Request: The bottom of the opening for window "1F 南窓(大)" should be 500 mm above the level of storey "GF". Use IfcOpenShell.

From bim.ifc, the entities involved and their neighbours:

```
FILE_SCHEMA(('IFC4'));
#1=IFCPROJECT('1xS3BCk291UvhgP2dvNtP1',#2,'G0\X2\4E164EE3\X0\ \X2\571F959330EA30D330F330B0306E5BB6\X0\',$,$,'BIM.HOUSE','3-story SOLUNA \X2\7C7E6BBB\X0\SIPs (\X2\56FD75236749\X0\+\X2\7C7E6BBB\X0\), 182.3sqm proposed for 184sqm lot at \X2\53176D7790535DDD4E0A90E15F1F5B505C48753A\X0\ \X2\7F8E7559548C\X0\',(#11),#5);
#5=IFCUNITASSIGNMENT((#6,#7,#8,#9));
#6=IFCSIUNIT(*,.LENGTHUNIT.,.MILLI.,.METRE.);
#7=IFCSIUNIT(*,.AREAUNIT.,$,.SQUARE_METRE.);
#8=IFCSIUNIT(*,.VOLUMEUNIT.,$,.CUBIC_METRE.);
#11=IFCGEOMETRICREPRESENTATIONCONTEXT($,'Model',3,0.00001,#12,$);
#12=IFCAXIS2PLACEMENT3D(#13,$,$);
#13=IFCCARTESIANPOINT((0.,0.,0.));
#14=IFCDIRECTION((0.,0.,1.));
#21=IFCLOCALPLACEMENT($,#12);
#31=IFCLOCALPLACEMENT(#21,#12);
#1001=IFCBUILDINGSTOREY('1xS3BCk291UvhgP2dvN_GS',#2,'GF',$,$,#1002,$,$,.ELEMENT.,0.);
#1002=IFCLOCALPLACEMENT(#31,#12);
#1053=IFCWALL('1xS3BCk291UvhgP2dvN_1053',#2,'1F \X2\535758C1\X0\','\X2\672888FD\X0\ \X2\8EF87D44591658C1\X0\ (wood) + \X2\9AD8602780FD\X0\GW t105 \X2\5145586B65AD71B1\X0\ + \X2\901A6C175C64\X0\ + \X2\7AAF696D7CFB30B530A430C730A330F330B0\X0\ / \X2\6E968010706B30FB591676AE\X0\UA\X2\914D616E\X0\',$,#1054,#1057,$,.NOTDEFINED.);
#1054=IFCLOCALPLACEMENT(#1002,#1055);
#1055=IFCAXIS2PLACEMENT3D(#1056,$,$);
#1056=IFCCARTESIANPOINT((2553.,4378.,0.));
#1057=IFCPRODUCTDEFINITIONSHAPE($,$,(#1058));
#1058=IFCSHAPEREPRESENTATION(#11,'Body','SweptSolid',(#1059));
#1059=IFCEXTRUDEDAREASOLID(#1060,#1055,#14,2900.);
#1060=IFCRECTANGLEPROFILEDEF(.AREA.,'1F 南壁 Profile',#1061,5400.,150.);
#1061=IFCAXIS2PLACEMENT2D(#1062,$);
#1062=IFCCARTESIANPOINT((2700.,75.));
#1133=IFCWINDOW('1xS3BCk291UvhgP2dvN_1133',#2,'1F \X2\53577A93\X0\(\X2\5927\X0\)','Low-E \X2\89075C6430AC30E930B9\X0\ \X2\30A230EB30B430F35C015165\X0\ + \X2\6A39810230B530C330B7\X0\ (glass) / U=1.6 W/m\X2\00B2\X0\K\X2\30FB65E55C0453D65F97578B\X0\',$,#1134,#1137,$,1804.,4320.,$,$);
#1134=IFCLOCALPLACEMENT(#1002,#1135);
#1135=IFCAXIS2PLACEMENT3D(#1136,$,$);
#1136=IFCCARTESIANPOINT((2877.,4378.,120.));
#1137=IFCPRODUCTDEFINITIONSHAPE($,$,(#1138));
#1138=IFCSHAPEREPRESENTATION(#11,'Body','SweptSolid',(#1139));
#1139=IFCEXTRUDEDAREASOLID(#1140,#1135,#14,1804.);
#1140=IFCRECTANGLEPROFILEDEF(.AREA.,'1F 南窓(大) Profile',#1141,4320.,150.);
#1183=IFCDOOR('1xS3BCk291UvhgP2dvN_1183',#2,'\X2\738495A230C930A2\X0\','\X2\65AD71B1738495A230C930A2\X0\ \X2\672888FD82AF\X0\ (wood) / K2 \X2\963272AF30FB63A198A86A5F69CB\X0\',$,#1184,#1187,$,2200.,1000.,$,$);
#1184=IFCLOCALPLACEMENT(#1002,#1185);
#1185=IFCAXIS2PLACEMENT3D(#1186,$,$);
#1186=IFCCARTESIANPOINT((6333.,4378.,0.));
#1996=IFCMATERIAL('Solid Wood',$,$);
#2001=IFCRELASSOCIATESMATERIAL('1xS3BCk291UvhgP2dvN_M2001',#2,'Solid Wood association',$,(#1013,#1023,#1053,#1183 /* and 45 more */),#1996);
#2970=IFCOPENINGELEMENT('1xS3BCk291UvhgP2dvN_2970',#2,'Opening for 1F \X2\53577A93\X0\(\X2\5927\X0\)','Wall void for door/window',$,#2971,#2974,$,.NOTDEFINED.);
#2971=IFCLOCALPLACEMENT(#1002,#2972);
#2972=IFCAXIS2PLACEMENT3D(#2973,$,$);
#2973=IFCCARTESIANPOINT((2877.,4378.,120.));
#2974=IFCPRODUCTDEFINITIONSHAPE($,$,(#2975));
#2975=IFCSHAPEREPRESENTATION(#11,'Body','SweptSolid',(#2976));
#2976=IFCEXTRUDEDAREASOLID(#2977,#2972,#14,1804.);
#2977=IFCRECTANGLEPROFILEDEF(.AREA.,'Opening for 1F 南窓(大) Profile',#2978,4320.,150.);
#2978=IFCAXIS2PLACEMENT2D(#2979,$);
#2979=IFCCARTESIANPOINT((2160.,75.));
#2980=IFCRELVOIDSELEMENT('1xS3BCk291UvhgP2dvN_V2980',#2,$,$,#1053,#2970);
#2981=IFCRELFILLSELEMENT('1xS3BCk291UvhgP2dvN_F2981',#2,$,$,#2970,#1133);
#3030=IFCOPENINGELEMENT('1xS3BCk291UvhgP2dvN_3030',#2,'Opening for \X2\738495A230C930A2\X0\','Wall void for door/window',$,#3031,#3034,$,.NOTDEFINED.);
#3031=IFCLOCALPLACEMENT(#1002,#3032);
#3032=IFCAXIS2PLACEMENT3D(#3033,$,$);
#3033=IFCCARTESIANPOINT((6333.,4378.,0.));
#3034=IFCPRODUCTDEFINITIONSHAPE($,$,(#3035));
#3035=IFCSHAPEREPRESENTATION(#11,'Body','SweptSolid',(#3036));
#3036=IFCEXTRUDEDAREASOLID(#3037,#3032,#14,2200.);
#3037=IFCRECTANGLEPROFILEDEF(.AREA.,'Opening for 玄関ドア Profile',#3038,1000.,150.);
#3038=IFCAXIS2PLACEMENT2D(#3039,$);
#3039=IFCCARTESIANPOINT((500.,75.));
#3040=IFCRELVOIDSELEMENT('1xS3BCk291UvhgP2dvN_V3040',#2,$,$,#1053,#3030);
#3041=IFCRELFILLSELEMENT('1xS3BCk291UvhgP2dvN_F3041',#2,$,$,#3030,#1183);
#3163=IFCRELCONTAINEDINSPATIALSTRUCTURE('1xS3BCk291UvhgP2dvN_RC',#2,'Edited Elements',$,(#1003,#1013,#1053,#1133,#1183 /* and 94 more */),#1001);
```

```python
import numpy as np
import ifcopenshell
import ifcopenshell.api.geometry
import ifcopenshell.geom
import ifcopenshell.util.element
import ifcopenshell.util.placement
import ifcopenshell.util.shape
import ifcopenshell.util.unit

model = ifcopenshell.open("bim.ifc")
unit_scale = ifcopenshell.util.unit.calculate_unit_scale(model)

window = model.by_guid("1xS3BCk291UvhgP2dvN_1133")
opening = window.FillsVoids[0].RelatingOpeningElement
storey = ifcopenshell.util.element.get_container(window, ifc_class="IfcBuildingStorey")
level = ifcopenshell.util.placement.get_local_placement(storey.ObjectPlacement)[2, 3]

# The opening's origin need not be at the sill, so measure its lowest point.
shape = ifcopenshell.geom.create_shape(ifcopenshell.geom.settings(), opening)
bottom = ifcopenshell.util.shape.get_shape_bottom_elevation(shape, shape.geometry) / unit_scale
dz = level + 0.5 / unit_scale - bottom

shift = np.array([0.0, 0.0, dz])
# The window is not placed relative to its opening, so move both.
for product in (opening, window):
    matrix = ifcopenshell.util.placement.get_local_placement(product.ObjectPlacement)
    matrix[:3, 3] += shift
    ifcopenshell.api.geometry.edit_object_placement(model, product=product, matrix=matrix, is_si=False)

print(f"moved by {dz * unit_scale:+.3f} m")

model.write("bim_edited.ifc")
```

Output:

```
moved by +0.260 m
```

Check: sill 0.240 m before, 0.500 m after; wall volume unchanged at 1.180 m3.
